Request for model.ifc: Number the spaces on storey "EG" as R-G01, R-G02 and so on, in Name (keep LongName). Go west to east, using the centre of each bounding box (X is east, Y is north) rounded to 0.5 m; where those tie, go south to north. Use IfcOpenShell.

First a look at what the model holds.

```python
import ifcopenshell
import ifcopenshell.util.element
import ifcopenshell.util.placement

model = ifcopenshell.open("model.ifc")
print(model.schema)
storey = next(s for s in model.by_type("IfcBuildingStorey") if s.Name == "EG")
spaces = [e for e in ifcopenshell.util.element.get_decomposition(storey) if e.is_a("IfcSpace")]
for e in sorted(spaces, key=lambda e: e.id()):
    origin = ifcopenshell.util.placement.get_local_placement(e.ObjectPlacement)[:3, 3]
    print(e.id(), e.Name, e.LongName, origin.round(2) + 0.0, sep=" | ")
```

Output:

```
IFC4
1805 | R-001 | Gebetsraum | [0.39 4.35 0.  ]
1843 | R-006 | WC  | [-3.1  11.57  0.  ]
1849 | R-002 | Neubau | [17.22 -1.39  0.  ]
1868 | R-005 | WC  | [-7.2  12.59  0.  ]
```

```python
import ifcopenshell
import ifcopenshell.geom
import ifcopenshell.util.element
import ifcopenshell.util.shape

model = ifcopenshell.open("model.ifc")
settings = ifcopenshell.geom.settings()
settings.set("use-world-coords", True)


def centre(element):
    shape = ifcopenshell.geom.create_shape(settings, element)
    return ifcopenshell.util.shape.get_bbox_centroid(shape.geometry)


storey = next(s for s in model.by_type("IfcBuildingStorey") if s.Name == "EG")
spaces = [e for e in ifcopenshell.util.element.get_decomposition(storey) if e.is_a("IfcSpace")]

# Insertion points can sit at a corner or the storey origin, so sort by the geometry (in metres).
centres = {e: centre(e) for e in spaces}
spaces.sort(key=lambda e: (round(centres[e][0] / 0.5), centres[e][1]))

for i, e in enumerate(spaces, start=1):
    number = f"R-G{i:02d}"
    e.Name = number
    print(e.id(), number)

model.write("model_rev.ifc")
```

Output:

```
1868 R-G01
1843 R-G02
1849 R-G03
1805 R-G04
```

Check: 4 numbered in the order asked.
